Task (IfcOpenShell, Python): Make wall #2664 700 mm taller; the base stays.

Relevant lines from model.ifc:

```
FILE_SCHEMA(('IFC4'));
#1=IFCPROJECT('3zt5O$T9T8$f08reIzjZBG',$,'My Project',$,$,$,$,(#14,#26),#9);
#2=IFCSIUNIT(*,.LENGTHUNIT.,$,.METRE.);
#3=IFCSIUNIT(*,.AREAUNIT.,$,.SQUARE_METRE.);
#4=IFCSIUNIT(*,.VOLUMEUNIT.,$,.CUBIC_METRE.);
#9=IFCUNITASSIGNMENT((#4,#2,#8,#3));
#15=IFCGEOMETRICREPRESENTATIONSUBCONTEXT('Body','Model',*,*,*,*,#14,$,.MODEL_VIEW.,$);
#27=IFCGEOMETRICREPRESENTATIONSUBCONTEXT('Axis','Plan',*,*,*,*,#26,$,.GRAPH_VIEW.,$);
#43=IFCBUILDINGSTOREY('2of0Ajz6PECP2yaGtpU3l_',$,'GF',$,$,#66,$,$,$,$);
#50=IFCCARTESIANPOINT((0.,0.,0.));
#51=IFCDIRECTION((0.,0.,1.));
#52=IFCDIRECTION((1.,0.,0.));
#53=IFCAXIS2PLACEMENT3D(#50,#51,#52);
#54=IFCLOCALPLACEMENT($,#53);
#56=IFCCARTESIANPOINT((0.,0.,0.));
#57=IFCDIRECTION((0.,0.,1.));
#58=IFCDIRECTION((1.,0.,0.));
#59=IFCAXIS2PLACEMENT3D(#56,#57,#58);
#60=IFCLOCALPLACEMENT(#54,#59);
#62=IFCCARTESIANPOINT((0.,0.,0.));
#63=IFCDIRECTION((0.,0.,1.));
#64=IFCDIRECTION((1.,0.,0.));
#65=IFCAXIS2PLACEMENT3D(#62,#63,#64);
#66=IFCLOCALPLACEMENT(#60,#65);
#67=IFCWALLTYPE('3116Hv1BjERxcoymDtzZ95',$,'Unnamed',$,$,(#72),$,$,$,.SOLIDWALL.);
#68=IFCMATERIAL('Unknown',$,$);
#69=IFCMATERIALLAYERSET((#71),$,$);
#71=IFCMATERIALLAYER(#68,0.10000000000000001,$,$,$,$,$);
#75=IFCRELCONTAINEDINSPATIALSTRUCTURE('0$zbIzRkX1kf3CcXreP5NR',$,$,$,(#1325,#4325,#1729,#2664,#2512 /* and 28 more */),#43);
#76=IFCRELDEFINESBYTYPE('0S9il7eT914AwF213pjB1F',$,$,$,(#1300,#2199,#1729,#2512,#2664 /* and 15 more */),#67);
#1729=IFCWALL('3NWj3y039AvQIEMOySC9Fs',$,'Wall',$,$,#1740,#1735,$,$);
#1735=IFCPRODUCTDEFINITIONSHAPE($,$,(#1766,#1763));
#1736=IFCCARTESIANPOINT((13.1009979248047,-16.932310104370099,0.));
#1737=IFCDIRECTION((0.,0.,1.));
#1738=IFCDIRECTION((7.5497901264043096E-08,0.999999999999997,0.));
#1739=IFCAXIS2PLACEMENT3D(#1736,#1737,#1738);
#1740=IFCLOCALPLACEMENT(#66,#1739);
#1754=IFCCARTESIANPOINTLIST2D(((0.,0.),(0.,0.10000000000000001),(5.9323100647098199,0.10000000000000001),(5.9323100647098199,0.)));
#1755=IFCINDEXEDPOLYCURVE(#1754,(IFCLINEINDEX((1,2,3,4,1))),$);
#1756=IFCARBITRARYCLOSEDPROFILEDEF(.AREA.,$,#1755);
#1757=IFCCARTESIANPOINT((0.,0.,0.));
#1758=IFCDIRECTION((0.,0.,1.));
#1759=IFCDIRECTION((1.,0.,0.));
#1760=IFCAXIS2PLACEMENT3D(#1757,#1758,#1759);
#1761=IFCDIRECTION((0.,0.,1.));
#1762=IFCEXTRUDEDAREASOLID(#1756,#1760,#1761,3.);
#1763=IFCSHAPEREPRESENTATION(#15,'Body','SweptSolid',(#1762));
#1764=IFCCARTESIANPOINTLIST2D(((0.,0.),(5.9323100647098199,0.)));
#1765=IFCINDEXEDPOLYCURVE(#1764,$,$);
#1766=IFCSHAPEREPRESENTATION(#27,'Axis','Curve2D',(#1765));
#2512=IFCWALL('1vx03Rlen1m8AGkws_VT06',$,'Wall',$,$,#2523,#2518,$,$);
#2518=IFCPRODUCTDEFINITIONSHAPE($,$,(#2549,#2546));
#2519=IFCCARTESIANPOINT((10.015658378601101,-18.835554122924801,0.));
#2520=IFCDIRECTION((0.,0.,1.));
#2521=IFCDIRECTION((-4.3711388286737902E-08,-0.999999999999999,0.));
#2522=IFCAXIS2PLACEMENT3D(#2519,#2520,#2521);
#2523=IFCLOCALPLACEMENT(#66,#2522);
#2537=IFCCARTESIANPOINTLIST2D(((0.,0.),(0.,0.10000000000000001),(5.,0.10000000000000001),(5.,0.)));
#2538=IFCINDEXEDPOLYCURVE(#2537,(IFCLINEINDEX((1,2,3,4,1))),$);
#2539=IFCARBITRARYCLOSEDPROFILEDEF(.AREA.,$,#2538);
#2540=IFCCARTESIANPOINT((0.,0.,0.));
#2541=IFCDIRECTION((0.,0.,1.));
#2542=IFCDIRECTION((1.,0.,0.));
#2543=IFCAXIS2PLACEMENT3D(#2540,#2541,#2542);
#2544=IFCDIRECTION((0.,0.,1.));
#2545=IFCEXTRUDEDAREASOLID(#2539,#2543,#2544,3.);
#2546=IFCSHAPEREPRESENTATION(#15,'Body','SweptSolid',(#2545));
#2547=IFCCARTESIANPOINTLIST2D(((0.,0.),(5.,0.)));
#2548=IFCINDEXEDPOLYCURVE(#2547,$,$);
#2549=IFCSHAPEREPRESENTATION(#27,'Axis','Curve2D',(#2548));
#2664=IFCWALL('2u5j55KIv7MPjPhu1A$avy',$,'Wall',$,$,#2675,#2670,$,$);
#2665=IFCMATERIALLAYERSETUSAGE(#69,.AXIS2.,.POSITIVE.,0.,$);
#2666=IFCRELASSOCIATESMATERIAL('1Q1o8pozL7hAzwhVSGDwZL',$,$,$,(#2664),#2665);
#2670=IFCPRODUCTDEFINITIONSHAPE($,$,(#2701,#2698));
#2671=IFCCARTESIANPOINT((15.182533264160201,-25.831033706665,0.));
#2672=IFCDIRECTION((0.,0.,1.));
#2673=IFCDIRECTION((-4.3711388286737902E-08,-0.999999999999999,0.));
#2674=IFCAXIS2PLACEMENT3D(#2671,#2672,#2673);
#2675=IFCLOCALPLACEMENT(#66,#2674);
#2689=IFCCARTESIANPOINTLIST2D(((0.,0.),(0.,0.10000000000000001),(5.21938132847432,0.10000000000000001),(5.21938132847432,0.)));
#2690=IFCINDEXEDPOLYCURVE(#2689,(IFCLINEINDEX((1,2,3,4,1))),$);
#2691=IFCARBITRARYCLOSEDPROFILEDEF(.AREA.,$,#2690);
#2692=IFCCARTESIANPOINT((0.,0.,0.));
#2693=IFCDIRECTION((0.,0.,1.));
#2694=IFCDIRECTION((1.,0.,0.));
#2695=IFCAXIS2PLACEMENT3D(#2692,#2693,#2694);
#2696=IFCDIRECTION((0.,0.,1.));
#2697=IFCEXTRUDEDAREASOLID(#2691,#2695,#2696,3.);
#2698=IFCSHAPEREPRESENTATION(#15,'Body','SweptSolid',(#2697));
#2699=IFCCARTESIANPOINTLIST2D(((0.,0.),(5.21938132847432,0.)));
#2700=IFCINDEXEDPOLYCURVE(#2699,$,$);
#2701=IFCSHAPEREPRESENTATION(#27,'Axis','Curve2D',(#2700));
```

```python
import ifcopenshell
import ifcopenshell.geom
import ifcopenshell.util.representation
import ifcopenshell.util.shape
import ifcopenshell.util.unit

model = ifcopenshell.open("model.ifc")
unit_scale = ifcopenshell.util.unit.calculate_unit_scale(model)
settings = ifcopenshell.geom.settings()


def volume(element):
    """Net volume in cubic metres, openings subtracted."""
    shape = ifcopenshell.geom.create_shape(settings, element)
    return ifcopenshell.util.shape.get_volume(shape.geometry)


wall = model.by_id(2664)
before = volume(wall)

body = ifcopenshell.util.representation.get_representation(wall, "Model", "Body")
solid = body.Items[0]
old_height = solid.Depth
solid.Depth += 0.7 / unit_scale
after = volume(wall)

print(f"height {old_height:g} -> {solid.Depth:g}, volume {before:.3f} -> {after:.3f} m3")

model.write("model-out.ifc")
```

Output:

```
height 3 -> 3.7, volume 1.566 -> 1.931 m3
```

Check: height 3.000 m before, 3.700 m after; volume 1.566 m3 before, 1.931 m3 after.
